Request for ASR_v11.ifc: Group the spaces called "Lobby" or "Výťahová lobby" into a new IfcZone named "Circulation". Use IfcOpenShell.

First a look at what the model holds.

```python
import ifcopenshell

model = ifcopenshell.open("ASR_v11.ifc")
print(model.schema)
seen = {}
for space in model.by_type("IfcSpace"):
    seen[space.LongName] = seen.get(space.LongName, 0) + 1
for name, count in sorted(seen.items(), key=str):
    print(count, "x", name)
print("zones:", [z.Name for z in model.by_type("IfcZone")][:20])
```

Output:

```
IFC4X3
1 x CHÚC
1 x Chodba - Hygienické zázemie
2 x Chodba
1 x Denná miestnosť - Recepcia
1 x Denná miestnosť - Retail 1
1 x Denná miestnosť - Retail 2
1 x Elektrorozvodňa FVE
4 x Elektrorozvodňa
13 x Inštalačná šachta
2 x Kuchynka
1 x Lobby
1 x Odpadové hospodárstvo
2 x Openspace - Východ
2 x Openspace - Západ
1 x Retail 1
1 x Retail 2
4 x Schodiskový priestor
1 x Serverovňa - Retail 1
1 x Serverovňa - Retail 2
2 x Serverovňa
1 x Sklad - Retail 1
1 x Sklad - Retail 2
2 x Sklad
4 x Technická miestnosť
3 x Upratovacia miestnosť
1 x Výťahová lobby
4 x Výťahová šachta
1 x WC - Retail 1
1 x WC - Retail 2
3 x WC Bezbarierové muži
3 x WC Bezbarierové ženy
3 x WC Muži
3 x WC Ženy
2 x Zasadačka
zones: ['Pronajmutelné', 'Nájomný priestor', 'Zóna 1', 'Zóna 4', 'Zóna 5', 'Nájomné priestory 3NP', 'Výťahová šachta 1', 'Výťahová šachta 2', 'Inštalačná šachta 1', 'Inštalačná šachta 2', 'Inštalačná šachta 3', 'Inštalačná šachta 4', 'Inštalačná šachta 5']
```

```python
import ifcopenshell
import ifcopenshell.api.group
import ifcopenshell.api.root

model = ifcopenshell.open("ASR_v11.ifc")

names = {"Lobby", "Výťahová lobby"}
spaces = [s for s in model.by_type("IfcSpace") if s.LongName in names]

zone = ifcopenshell.api.root.create_entity(model, ifc_class="IfcZone", name="Circulation")
ifcopenshell.api.group.assign_group(model, products=spaces, group=zone)
print(len(spaces), "spaces in", zone.Name)

model.write("ASR_v11_updated.ifc")
```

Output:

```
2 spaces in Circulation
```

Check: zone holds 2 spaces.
